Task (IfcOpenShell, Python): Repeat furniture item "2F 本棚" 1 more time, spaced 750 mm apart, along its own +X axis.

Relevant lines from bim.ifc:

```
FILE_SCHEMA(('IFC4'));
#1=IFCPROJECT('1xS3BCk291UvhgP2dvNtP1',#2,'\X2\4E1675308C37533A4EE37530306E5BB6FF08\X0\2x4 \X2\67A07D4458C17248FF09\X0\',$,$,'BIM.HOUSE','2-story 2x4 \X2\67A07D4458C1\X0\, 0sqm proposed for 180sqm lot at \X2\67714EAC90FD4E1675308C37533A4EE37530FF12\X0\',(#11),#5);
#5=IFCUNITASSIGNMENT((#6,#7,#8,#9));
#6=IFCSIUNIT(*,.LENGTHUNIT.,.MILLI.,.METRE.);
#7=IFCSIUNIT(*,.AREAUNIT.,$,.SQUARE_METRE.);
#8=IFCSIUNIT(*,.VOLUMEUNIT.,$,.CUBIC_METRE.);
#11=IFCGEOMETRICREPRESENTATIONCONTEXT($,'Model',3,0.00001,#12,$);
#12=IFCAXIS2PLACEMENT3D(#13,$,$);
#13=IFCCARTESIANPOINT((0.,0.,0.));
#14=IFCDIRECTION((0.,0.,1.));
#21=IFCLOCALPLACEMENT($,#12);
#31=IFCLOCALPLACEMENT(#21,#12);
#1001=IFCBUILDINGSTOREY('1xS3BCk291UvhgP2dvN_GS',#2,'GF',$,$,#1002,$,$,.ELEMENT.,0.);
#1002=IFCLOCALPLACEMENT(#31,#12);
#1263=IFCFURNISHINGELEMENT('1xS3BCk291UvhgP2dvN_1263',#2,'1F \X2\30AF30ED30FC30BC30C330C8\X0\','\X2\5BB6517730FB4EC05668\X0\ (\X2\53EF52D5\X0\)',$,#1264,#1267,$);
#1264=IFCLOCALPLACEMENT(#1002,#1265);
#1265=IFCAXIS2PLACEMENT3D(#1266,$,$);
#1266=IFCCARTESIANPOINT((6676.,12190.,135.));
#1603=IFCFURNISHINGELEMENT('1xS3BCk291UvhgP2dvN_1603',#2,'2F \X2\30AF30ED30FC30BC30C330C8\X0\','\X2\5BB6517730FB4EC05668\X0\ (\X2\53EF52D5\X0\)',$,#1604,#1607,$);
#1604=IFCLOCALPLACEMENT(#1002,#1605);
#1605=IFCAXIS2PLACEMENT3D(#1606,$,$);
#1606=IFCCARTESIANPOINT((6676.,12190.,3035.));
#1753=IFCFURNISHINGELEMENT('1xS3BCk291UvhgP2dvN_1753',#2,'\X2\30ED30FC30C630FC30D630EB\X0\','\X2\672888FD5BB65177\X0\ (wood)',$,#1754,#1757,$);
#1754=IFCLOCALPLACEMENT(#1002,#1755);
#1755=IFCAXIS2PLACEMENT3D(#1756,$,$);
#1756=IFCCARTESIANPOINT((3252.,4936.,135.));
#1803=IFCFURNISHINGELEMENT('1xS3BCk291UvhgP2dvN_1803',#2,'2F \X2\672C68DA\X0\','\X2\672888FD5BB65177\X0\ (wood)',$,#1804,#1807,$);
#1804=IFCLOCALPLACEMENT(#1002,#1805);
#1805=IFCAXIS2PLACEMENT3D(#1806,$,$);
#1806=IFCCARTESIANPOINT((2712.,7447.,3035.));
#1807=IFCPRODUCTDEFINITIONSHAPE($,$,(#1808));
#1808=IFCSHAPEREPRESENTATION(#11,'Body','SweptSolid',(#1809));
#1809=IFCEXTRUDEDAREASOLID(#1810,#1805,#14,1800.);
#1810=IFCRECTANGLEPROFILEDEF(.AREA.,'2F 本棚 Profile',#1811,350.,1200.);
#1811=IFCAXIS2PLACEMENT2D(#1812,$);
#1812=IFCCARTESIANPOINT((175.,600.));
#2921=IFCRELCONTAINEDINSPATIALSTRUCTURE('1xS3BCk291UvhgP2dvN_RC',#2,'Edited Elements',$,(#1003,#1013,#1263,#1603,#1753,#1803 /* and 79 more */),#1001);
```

```python
import ifcopenshell
import ifcopenshell.api.geometry
import ifcopenshell.api.root
import ifcopenshell.util.element
import ifcopenshell.util.placement

model = ifcopenshell.open("bim.ifc")


def reuse_history(source, copy):
    """copy_class also copies each property set's owner history, people and application; keep the originals."""
    for rel in copy.IsDefinedBy:
        if rel.is_a("IfcRelDefinesByProperties") and (history := rel.RelatingPropertyDefinition.OwnerHistory):
            rel.RelatingPropertyDefinition.OwnerHistory = source.OwnerHistory
            ifcopenshell.util.element.remove_deep2(model, history)


source = model.by_guid("1xS3BCk291UvhgP2dvN_1803")
base = ifcopenshell.util.placement.get_local_placement(source.ObjectPlacement)
step = base[:3, 0] * 750.0

for i in range(1, 2):
    copy = ifcopenshell.api.root.copy_class(model, product=source)
    copy.Representation = ifcopenshell.util.element.copy_deep(
        model, source.Representation, exclude=["IfcGeometricRepresentationContext", "IfcRepresentationMap"]
    )
    reuse_history(source, copy)
    matrix = base.copy()
    matrix[:3, 3] += i * step
    print("added at", matrix[:3, 3].round(3) + 0.0)
    ifcopenshell.api.geometry.edit_object_placement(model, product=copy, matrix=matrix, is_si=False)

model.write("bim_v2.ifc")
```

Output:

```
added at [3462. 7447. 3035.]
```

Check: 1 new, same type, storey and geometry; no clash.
